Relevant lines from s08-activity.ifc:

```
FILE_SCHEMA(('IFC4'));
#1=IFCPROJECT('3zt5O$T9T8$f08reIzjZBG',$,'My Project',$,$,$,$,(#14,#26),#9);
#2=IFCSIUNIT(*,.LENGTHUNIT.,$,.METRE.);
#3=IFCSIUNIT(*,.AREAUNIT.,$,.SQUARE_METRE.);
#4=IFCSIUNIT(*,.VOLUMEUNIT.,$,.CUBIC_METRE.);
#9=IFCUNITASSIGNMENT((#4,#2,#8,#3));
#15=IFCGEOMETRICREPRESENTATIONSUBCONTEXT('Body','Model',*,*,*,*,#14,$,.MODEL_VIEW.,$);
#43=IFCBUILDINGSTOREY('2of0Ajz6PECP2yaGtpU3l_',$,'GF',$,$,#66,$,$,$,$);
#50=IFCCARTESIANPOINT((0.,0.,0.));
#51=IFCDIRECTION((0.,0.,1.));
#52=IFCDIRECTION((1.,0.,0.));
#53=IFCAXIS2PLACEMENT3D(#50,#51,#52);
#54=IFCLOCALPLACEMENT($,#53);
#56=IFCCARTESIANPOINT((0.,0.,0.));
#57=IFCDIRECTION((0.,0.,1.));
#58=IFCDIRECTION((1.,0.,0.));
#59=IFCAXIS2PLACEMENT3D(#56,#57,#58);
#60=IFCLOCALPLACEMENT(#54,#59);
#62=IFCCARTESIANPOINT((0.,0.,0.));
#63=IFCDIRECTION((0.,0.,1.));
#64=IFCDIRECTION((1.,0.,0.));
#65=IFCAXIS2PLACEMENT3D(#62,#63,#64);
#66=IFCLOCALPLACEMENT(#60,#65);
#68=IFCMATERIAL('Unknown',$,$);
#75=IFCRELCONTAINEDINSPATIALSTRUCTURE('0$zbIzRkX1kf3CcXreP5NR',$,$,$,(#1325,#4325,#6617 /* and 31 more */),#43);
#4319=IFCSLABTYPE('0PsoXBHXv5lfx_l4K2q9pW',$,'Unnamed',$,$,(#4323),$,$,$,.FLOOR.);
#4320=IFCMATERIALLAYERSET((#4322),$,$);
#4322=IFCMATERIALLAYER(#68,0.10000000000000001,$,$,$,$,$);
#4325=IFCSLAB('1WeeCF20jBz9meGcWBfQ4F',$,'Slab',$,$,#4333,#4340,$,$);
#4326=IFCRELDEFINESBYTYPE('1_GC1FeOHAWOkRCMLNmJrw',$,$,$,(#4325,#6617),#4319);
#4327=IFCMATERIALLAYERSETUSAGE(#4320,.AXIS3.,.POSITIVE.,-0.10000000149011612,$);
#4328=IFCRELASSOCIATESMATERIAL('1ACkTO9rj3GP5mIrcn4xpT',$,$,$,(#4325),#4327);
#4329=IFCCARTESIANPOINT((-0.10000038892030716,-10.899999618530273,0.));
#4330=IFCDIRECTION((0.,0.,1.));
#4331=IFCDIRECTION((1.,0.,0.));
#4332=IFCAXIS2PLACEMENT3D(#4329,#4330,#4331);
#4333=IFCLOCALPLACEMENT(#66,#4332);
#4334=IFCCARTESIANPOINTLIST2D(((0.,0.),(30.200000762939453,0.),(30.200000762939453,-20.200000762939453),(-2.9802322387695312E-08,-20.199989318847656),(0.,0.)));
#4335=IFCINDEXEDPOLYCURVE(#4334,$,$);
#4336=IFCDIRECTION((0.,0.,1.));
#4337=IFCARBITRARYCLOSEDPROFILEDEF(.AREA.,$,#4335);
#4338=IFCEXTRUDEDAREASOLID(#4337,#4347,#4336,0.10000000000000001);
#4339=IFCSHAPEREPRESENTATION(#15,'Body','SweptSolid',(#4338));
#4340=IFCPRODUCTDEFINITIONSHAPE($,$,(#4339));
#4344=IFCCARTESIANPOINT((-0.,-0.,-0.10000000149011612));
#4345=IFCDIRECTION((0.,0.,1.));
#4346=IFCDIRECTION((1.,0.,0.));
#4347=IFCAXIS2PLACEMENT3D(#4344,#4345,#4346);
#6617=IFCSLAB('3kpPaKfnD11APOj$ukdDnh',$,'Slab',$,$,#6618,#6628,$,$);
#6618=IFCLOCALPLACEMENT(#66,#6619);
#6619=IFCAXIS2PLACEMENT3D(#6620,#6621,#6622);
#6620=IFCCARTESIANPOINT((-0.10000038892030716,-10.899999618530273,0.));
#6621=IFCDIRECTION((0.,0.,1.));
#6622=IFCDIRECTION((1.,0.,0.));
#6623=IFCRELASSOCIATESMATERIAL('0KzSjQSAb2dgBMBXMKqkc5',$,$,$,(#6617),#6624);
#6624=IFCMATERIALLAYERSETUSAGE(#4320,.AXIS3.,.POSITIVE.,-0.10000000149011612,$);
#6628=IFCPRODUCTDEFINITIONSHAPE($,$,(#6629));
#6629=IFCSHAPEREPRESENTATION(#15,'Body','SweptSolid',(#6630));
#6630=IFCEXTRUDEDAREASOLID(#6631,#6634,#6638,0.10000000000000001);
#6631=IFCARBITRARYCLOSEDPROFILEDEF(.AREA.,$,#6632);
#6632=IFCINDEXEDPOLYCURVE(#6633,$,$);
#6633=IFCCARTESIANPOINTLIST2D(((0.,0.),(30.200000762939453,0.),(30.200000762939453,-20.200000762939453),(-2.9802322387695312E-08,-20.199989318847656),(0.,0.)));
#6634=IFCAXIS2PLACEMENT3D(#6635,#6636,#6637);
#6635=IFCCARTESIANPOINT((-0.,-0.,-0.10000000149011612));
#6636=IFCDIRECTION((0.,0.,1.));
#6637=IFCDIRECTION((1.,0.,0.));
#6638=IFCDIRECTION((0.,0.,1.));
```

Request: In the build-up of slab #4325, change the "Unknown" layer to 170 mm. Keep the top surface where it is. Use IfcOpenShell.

```python
import ifcopenshell
import ifcopenshell.util.element
import ifcopenshell.util.representation

model = ifcopenshell.open("s08-activity.ifc")

layer_set = model.by_id(4320)
layer = next(l for l in layer_set.MaterialLayers if l.Material and l.Material.Name == "Unknown")
change = 0.17 - layer.LayerThickness
layer.LayerThickness += change

# The layer set is shared, so every slab that uses it gets the new thickness.
slabs = [e for e in ifcopenshell.util.element.get_elements_by_material(model, layer_set) if e.is_a("IfcSlab")]
for slab in sorted(slabs, key=lambda e: e.id()):
    body = ifcopenshell.util.representation.get_representation(slab, "Model", "Body")
    solid = body.Items[0]
    old_depth = solid.Depth
    solid.Depth += change
    # Extruded upwards: lower the start of the extrusion so the top stays.
    x, y, z = solid.Position.Location.Coordinates
    solid.Position.Location = model.createIfcCartesianPoint((x, y, z - change))
    print(slab.id(), f"{old_depth:g} -> {solid.Depth:g}")

# The layers are counted up from the underside, which has moved.
for usage in {ifcopenshell.util.element.get_material(slab) for slab in slabs}:
    usage.OffsetFromReferenceLine -= change

model.write("s08-activity_v2.ifc")
```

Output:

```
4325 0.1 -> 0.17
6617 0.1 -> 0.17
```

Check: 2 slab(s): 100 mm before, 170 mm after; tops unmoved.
